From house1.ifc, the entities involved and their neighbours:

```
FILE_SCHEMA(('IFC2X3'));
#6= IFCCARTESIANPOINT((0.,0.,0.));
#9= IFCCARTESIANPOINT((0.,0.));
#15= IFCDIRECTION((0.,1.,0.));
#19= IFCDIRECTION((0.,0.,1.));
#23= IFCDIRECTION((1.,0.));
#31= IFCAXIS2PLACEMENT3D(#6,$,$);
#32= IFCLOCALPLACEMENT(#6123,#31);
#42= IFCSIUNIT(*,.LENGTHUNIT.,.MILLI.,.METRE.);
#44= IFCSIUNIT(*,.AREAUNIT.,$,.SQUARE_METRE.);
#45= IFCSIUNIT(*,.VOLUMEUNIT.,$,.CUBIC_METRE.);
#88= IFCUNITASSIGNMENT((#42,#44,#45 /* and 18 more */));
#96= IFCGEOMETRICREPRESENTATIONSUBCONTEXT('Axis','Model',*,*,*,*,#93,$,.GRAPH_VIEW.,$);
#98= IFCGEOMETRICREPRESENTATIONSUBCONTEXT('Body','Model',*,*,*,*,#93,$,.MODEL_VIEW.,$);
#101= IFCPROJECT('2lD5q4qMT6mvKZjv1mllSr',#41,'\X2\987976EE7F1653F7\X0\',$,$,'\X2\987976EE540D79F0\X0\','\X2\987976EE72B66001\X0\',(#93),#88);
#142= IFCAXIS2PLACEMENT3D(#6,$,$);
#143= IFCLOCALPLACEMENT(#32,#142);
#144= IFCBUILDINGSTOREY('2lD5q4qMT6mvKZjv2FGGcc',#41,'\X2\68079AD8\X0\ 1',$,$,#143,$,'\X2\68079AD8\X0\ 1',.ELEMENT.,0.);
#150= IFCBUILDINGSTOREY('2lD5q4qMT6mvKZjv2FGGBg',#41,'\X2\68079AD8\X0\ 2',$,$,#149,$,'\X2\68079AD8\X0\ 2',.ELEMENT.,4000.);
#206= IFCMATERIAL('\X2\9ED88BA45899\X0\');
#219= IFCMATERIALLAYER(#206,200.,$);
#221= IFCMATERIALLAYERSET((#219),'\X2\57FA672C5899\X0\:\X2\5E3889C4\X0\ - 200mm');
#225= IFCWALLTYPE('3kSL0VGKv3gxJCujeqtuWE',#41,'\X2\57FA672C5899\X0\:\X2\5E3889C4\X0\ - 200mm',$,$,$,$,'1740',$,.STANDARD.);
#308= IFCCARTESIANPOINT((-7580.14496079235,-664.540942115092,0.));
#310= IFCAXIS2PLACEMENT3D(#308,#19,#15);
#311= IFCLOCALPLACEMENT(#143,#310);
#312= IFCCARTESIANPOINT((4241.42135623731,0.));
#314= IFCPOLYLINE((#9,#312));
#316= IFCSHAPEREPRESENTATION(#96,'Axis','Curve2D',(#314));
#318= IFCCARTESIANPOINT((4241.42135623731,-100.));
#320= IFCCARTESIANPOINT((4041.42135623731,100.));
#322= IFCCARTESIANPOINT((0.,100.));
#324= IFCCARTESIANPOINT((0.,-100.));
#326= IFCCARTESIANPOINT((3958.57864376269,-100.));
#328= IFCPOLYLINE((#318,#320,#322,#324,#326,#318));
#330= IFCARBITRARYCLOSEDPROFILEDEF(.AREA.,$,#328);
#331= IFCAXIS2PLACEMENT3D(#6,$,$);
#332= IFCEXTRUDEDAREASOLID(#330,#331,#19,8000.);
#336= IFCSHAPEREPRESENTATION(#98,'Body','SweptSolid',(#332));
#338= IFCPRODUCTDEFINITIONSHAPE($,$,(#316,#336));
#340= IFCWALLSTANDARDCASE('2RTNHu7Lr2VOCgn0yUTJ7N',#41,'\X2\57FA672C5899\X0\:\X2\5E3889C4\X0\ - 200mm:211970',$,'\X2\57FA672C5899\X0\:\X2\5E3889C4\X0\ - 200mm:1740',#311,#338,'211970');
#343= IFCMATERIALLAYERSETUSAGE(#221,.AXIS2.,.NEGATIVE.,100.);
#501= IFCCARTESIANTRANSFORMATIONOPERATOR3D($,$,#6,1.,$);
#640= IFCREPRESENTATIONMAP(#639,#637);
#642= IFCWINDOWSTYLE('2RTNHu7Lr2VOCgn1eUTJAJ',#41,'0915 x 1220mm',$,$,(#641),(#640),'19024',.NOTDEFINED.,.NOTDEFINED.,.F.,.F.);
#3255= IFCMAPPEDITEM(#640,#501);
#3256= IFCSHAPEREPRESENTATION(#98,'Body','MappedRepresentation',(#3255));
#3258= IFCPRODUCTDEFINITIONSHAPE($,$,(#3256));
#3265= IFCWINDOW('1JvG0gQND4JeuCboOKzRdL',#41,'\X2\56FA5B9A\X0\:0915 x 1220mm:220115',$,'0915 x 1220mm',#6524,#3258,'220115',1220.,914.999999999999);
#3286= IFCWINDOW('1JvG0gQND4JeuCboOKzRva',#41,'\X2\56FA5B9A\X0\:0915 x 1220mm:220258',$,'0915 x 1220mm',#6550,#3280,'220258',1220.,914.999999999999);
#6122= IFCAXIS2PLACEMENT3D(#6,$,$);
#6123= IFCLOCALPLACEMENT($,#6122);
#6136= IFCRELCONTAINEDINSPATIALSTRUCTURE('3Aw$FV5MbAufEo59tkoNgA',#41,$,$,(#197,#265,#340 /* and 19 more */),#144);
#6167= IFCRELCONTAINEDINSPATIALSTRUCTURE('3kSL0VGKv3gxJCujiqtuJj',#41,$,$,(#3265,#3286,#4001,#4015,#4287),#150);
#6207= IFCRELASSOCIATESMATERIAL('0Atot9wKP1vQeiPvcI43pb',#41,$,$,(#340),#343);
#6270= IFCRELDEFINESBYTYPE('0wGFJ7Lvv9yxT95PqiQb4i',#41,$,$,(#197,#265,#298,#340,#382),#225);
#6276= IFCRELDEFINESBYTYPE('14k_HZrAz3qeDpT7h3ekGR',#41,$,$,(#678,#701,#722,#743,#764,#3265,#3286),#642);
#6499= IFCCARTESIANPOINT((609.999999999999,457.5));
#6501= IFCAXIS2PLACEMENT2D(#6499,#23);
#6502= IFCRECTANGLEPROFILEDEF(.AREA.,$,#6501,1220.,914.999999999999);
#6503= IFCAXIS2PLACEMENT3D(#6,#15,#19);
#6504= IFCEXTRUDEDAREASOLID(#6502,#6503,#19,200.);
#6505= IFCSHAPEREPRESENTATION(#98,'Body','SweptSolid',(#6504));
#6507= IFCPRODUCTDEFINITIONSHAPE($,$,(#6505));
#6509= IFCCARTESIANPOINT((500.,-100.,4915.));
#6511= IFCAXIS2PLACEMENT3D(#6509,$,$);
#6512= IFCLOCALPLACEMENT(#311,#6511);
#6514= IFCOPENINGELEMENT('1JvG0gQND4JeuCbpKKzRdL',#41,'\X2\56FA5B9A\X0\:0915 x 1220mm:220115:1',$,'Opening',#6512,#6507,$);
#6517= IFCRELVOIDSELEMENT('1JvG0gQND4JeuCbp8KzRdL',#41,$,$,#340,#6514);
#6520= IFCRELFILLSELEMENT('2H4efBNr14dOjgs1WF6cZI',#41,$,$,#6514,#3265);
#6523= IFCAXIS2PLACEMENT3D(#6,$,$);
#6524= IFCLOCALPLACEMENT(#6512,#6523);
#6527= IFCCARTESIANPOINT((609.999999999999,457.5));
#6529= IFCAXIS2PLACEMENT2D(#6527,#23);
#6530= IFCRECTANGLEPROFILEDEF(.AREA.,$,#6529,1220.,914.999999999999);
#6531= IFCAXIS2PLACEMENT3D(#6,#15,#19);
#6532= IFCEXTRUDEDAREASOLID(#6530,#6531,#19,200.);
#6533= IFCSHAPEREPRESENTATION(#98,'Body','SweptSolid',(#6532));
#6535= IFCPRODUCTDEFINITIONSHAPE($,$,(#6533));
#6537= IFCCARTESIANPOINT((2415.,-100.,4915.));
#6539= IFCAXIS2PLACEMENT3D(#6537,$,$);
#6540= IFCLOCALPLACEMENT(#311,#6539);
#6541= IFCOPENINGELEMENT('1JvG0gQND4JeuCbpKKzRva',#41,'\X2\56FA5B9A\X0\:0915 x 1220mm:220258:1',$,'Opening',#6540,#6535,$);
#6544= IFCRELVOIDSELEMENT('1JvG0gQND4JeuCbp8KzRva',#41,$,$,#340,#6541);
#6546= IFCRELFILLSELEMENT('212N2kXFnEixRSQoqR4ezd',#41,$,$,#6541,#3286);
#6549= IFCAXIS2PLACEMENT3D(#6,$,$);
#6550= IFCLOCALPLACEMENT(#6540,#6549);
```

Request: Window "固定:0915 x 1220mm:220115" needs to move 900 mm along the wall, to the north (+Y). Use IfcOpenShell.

```python
import ifcopenshell
import ifcopenshell.api.geometry
import ifcopenshell.util.placement

model = ifcopenshell.open("house1.ifc")

window = model.by_guid("1JvG0gQND4JeuCboOKzRdL")
opening = window.FillsVoids[0].RelatingOpeningElement
wall = opening.VoidsElements[0].RelatingBuildingElement

wall_matrix = ifcopenshell.util.placement.get_local_placement(wall.ObjectPlacement)
shift = wall_matrix[:3, 0] * 900.0
before = ifcopenshell.util.placement.get_local_placement(window.ObjectPlacement)[:3, 3].copy()

# The window is placed relative to its opening, so it follows when the opening moves.
matrix = ifcopenshell.util.placement.get_local_placement(opening.ObjectPlacement)
matrix[:3, 3] += shift
ifcopenshell.api.geometry.edit_object_placement(
    model, product=opening, matrix=matrix, is_si=False, should_transform_children=True
)

after = ifcopenshell.util.placement.get_local_placement(window.ObjectPlacement)[:3, 3]
print("window moved by", (after - before).round(3) + 0.0)

model.write("house1_edited.ifc")
```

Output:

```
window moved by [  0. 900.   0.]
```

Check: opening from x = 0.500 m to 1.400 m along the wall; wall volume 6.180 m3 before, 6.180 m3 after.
